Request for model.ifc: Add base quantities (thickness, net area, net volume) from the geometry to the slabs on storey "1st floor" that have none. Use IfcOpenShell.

First a look at what the model holds.

```python
import ifcopenshell
import ifcopenshell.util.element
import ifcopenshell.util.unit

model = ifcopenshell.open("model.ifc")
print(model.schema)
for unit_type in ("LENGTHUNIT", "AREAUNIT", "VOLUMEUNIT"):
    print(unit_type, ifcopenshell.util.unit.calculate_unit_scale(model, unit_type))
storey = next(s for s in model.by_type("IfcBuildingStorey") if s.Name == "1st floor")
slabs = [e for e in ifcopenshell.util.element.get_decomposition(storey) if e.is_a("IfcSlab")]
for e in sorted(slabs, key=lambda e: e.id()):
    print(e.id(), e.is_a(), e.Name, list(ifcopenshell.util.element.get_psets(e, qtos_only=True)), sep=" | ")
```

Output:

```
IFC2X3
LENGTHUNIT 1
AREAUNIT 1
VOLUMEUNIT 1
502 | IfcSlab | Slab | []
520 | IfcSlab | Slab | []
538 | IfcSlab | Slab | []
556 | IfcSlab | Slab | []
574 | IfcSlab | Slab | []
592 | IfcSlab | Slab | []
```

```python
import ifcopenshell
import ifcopenshell.api.pset
import ifcopenshell.geom
import ifcopenshell.util.element
import ifcopenshell.util.shape
import ifcopenshell.util.unit

model = ifcopenshell.open("model.ifc")
unit_scale = ifcopenshell.util.unit.calculate_unit_scale(model)
area_scale = ifcopenshell.util.unit.calculate_unit_scale(model, "AREAUNIT")
volume_scale = ifcopenshell.util.unit.calculate_unit_scale(model, "VOLUMEUNIT")
settings = ifcopenshell.geom.settings()

storey = next(s for s in model.by_type("IfcBuildingStorey") if s.Name == "1st floor")
slabs = [e for e in ifcopenshell.util.element.get_decomposition(storey) if e.is_a("IfcSlab")]

for e in sorted(slabs, key=lambda e: e.id()):
    if ifcopenshell.util.element.get_psets(e, qtos_only=True, should_inherit=False):
        continue
    # Geometry comes back in metres, in the element's own axes.
    shape = ifcopenshell.geom.create_shape(settings, e)
    values = {
        "Width": ifcopenshell.util.shape.get_z(shape.geometry) / unit_scale,
        "NetArea": ifcopenshell.util.shape.get_footprint_area(shape.geometry) / area_scale,
        "NetVolume": ifcopenshell.util.shape.get_volume(shape.geometry) / volume_scale,
    }
    qto = ifcopenshell.api.pset.add_qto(model, product=e, name="BaseQuantities")
    ifcopenshell.api.pset.edit_qto(model, qto=qto, properties=values)
    print(e.id(), {k: round(v, 3) for k, v in values.items()})

model.write("model_updated.ifc")
```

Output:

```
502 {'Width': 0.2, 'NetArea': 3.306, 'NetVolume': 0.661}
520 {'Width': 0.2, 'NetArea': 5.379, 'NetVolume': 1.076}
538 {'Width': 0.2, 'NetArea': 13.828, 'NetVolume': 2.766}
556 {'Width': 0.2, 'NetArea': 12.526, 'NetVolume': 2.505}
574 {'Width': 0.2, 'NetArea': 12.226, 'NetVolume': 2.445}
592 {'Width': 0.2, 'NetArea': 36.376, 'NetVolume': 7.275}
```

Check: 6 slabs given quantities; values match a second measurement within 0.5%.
